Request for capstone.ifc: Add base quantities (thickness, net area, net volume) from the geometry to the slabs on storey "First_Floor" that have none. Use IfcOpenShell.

First a look at what the model holds.

```python
import ifcopenshell
import ifcopenshell.util.element
import ifcopenshell.util.unit

model = ifcopenshell.open("capstone.ifc")
print(model.schema)
for unit_type in ("LENGTHUNIT", "AREAUNIT", "VOLUMEUNIT"):
    print(unit_type, ifcopenshell.util.unit.calculate_unit_scale(model, unit_type))
storey = next(s for s in model.by_type("IfcBuildingStorey") if s.Name == "First_Floor")
slabs = [e for e in ifcopenshell.util.element.get_decomposition(storey) if e.is_a("IfcSlab")]
for e in sorted(slabs, key=lambda e: e.id()):
    print(e.id(), e.is_a(), e.Name, list(ifcopenshell.util.element.get_psets(e, qtos_only=True)), sep=" | ")
```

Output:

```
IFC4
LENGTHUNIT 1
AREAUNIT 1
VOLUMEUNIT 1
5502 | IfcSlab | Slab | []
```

```python
import ifcopenshell
import ifcopenshell.api.pset
import ifcopenshell.geom
import ifcopenshell.util.element
import ifcopenshell.util.shape
import ifcopenshell.util.unit

model = ifcopenshell.open("capstone.ifc")
unit_scale = ifcopenshell.util.unit.calculate_unit_scale(model)
area_scale = ifcopenshell.util.unit.calculate_unit_scale(model, "AREAUNIT")
volume_scale = ifcopenshell.util.unit.calculate_unit_scale(model, "VOLUMEUNIT")
settings = ifcopenshell.geom.settings()

storey = next(s for s in model.by_type("IfcBuildingStorey") if s.Name == "First_Floor")
slabs = [e for e in ifcopenshell.util.element.get_decomposition(storey) if e.is_a("IfcSlab")]

for e in sorted(slabs, key=lambda e: e.id()):
    if ifcopenshell.util.element.get_psets(e, qtos_only=True, should_inherit=False):
        continue
    # Geometry comes back in metres, in the element's own axes.
    shape = ifcopenshell.geom.create_shape(settings, e)
    values = {
        "Width": ifcopenshell.util.shape.get_z(shape.geometry) / unit_scale,
        "NetArea": ifcopenshell.util.shape.get_footprint_area(shape.geometry) / area_scale,
        "NetVolume": ifcopenshell.util.shape.get_volume(shape.geometry) / volume_scale,
    }
    qto = ifcopenshell.api.pset.add_qto(model, product=e, name="Qto_SlabBaseQuantities")
    ifcopenshell.api.pset.edit_qto(model, qto=qto, properties=values)
    print(e.id(), {k: round(v, 3) for k, v in values.items()})

model.write("capstone-out.ifc")
```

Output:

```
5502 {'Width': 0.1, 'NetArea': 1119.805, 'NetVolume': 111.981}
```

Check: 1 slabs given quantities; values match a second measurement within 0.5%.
